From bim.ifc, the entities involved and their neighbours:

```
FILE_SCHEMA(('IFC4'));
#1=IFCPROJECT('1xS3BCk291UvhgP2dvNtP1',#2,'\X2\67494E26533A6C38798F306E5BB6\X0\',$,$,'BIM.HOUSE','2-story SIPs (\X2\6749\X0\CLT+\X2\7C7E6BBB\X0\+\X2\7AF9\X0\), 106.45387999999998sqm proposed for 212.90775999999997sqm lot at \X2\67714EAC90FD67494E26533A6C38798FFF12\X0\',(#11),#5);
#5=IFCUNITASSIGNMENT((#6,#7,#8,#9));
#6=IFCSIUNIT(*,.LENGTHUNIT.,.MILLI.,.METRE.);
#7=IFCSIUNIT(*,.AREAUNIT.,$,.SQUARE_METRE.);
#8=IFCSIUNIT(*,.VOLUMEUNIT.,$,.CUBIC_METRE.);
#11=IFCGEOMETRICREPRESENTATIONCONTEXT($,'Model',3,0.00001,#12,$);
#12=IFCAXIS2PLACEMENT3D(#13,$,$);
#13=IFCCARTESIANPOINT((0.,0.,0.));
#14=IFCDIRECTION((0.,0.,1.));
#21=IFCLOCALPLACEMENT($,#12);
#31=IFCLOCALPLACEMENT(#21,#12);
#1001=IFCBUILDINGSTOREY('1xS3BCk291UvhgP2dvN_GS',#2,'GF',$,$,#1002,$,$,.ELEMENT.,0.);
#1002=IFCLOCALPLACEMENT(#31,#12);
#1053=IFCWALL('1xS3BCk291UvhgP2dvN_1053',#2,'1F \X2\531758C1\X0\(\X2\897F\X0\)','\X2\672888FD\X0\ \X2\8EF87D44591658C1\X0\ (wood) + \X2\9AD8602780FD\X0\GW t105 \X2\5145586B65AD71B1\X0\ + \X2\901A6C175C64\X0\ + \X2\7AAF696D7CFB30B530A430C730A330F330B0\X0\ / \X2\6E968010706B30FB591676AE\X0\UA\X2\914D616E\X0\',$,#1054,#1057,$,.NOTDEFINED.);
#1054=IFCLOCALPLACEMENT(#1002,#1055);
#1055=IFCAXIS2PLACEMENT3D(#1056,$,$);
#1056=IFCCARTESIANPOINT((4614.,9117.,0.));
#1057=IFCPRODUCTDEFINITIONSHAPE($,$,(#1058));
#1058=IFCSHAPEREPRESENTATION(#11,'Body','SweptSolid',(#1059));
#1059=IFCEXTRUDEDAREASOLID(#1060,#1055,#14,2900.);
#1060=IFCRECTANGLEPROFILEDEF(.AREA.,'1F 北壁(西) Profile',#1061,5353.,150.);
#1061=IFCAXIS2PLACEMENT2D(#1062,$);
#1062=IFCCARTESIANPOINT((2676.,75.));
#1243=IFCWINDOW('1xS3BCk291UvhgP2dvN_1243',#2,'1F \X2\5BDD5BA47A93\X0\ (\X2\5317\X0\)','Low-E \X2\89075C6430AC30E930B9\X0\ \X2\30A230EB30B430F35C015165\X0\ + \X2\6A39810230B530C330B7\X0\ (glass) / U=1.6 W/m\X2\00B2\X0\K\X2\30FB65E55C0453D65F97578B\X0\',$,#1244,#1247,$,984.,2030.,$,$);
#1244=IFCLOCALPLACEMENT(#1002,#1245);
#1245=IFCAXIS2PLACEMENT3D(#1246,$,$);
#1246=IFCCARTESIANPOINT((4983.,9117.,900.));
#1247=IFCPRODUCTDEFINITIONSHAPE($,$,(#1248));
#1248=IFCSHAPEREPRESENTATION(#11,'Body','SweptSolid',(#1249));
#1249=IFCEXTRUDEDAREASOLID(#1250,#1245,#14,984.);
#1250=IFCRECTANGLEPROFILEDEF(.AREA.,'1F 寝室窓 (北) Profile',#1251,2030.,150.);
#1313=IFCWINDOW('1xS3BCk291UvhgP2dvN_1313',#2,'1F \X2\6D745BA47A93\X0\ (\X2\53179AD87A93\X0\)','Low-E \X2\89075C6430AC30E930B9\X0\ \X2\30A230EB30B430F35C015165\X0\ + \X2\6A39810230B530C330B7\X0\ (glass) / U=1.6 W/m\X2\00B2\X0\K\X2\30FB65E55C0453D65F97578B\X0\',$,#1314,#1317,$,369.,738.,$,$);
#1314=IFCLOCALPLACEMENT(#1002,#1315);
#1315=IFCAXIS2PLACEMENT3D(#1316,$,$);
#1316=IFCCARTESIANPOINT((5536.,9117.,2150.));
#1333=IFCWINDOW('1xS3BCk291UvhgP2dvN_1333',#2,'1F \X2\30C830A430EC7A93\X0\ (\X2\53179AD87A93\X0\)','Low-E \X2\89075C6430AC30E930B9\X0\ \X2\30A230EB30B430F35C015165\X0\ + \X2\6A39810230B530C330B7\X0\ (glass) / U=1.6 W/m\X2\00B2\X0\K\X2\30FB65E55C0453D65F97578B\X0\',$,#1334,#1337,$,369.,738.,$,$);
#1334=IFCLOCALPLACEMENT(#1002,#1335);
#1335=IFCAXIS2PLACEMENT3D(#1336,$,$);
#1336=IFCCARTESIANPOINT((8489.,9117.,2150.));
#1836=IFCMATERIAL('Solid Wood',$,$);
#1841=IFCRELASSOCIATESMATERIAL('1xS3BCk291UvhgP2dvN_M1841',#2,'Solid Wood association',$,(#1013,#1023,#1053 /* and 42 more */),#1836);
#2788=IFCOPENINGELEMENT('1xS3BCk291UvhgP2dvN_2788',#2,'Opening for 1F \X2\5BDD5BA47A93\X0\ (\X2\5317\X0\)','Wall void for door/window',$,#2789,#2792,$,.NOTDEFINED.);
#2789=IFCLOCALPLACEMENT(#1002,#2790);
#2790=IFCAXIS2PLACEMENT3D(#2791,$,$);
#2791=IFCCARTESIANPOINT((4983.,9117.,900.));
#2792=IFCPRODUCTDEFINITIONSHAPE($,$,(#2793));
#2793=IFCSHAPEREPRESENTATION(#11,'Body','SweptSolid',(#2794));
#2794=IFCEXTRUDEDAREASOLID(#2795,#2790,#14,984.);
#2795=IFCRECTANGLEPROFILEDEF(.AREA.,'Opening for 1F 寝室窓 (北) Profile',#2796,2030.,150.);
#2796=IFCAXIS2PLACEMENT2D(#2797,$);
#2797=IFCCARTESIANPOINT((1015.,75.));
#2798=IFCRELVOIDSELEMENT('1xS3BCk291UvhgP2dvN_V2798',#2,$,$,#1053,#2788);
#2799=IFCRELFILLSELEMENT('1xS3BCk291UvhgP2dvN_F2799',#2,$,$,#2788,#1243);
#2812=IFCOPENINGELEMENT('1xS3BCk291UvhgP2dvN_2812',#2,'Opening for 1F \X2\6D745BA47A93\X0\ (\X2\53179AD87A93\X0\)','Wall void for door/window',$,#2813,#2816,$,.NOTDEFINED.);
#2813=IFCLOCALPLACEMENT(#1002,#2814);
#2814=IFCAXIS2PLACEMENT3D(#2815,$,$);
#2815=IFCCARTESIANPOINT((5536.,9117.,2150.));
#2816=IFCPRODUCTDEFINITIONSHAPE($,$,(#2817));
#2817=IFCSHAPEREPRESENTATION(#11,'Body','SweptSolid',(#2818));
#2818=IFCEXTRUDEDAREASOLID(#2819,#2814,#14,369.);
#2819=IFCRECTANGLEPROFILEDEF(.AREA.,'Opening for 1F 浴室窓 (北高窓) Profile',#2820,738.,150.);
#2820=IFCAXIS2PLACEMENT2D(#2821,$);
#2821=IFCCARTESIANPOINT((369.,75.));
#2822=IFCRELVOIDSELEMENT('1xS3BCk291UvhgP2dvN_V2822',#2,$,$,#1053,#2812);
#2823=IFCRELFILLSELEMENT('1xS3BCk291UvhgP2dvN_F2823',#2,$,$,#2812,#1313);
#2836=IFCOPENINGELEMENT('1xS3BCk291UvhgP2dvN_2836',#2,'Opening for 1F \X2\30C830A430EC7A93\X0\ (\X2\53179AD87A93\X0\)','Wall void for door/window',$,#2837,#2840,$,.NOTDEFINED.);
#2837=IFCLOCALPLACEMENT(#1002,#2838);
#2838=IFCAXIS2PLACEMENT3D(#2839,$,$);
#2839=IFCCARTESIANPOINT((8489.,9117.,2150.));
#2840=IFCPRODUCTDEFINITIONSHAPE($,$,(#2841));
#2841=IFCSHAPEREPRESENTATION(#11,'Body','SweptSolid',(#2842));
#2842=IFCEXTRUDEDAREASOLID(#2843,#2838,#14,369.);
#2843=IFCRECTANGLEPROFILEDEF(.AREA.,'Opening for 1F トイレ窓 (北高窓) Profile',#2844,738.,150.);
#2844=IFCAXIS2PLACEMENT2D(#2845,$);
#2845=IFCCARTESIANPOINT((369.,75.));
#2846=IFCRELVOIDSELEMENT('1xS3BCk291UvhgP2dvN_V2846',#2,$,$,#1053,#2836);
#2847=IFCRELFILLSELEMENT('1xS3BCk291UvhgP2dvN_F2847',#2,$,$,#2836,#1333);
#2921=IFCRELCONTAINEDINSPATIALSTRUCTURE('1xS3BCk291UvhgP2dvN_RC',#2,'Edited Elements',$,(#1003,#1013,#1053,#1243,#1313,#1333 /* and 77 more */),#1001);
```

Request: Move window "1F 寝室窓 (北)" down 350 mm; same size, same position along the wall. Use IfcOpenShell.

```python
import numpy as np
import ifcopenshell
import ifcopenshell.api.geometry
import ifcopenshell.util.placement
import ifcopenshell.util.unit

model = ifcopenshell.open("bim.ifc")
unit_scale = ifcopenshell.util.unit.calculate_unit_scale(model)

window = model.by_guid("1xS3BCk291UvhgP2dvN_1243")
opening = window.FillsVoids[0].RelatingOpeningElement
dz = -0.35 / unit_scale

shift = np.array([0.0, 0.0, dz])
# The window is not placed relative to its opening, so move both.
for product in (opening, window):
    matrix = ifcopenshell.util.placement.get_local_placement(product.ObjectPlacement)
    matrix[:3, 3] += shift
    ifcopenshell.api.geometry.edit_object_placement(model, product=product, matrix=matrix, is_si=False)

print(f"moved by {dz * unit_scale:+.3f} m")

model.write("bim_v2.ifc")
```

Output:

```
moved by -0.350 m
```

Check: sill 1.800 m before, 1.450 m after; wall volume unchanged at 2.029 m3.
